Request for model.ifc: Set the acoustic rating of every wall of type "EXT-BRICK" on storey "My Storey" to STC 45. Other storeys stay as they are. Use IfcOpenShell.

First a look at what the model holds.

```python
import ifcopenshell
import ifcopenshell.util.element

model = ifcopenshell.open("model.ifc")
print(model.schema)
storey = next(s for s in model.by_type("IfcBuildingStorey") if s.Name == "My Storey")
walls = [e for e in ifcopenshell.util.element.get_decomposition(storey) if e.is_a("IfcWall")]
seen = {}
for e in walls:
    element_type = ifcopenshell.util.element.get_type(e)
    key = (element_type.Name if element_type != e and element_type else None, ifcopenshell.util.element.get_pset(e, "Pset_WallCommon", "AcousticRating"))
    seen[key] = seen.get(key, 0) + 1
for (name, value), count in sorted(seen.items(), key=str):
    print(count, "x", name, "|", value)
```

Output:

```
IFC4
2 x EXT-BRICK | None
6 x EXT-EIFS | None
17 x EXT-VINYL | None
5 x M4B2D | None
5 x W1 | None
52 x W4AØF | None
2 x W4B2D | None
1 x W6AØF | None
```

```python
import ifcopenshell
import ifcopenshell.api.pset
import ifcopenshell.util.element

model = ifcopenshell.open("model.ifc")

storey = next(s for s in model.by_type("IfcBuildingStorey") if s.Name == "My Storey")
walls = [e for e in ifcopenshell.util.element.get_decomposition(storey) if e.is_a("IfcWall")]

count = 0
for e in walls:
    element_type = ifcopenshell.util.element.get_type(e)
    if element_type in (None, e) or element_type.Name != "EXT-BRICK":
        continue
    # add_pset returns the element's existing set when there is one.
    pset = ifcopenshell.api.pset.add_pset(model, product=e, name="Pset_WallCommon")
    ifcopenshell.api.pset.edit_pset(model, pset=pset, properties={"AcousticRating": "STC 45"})
    count += 1

print(count, "walls updated")

model.write("model-out.ifc")
```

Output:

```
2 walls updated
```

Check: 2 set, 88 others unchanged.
